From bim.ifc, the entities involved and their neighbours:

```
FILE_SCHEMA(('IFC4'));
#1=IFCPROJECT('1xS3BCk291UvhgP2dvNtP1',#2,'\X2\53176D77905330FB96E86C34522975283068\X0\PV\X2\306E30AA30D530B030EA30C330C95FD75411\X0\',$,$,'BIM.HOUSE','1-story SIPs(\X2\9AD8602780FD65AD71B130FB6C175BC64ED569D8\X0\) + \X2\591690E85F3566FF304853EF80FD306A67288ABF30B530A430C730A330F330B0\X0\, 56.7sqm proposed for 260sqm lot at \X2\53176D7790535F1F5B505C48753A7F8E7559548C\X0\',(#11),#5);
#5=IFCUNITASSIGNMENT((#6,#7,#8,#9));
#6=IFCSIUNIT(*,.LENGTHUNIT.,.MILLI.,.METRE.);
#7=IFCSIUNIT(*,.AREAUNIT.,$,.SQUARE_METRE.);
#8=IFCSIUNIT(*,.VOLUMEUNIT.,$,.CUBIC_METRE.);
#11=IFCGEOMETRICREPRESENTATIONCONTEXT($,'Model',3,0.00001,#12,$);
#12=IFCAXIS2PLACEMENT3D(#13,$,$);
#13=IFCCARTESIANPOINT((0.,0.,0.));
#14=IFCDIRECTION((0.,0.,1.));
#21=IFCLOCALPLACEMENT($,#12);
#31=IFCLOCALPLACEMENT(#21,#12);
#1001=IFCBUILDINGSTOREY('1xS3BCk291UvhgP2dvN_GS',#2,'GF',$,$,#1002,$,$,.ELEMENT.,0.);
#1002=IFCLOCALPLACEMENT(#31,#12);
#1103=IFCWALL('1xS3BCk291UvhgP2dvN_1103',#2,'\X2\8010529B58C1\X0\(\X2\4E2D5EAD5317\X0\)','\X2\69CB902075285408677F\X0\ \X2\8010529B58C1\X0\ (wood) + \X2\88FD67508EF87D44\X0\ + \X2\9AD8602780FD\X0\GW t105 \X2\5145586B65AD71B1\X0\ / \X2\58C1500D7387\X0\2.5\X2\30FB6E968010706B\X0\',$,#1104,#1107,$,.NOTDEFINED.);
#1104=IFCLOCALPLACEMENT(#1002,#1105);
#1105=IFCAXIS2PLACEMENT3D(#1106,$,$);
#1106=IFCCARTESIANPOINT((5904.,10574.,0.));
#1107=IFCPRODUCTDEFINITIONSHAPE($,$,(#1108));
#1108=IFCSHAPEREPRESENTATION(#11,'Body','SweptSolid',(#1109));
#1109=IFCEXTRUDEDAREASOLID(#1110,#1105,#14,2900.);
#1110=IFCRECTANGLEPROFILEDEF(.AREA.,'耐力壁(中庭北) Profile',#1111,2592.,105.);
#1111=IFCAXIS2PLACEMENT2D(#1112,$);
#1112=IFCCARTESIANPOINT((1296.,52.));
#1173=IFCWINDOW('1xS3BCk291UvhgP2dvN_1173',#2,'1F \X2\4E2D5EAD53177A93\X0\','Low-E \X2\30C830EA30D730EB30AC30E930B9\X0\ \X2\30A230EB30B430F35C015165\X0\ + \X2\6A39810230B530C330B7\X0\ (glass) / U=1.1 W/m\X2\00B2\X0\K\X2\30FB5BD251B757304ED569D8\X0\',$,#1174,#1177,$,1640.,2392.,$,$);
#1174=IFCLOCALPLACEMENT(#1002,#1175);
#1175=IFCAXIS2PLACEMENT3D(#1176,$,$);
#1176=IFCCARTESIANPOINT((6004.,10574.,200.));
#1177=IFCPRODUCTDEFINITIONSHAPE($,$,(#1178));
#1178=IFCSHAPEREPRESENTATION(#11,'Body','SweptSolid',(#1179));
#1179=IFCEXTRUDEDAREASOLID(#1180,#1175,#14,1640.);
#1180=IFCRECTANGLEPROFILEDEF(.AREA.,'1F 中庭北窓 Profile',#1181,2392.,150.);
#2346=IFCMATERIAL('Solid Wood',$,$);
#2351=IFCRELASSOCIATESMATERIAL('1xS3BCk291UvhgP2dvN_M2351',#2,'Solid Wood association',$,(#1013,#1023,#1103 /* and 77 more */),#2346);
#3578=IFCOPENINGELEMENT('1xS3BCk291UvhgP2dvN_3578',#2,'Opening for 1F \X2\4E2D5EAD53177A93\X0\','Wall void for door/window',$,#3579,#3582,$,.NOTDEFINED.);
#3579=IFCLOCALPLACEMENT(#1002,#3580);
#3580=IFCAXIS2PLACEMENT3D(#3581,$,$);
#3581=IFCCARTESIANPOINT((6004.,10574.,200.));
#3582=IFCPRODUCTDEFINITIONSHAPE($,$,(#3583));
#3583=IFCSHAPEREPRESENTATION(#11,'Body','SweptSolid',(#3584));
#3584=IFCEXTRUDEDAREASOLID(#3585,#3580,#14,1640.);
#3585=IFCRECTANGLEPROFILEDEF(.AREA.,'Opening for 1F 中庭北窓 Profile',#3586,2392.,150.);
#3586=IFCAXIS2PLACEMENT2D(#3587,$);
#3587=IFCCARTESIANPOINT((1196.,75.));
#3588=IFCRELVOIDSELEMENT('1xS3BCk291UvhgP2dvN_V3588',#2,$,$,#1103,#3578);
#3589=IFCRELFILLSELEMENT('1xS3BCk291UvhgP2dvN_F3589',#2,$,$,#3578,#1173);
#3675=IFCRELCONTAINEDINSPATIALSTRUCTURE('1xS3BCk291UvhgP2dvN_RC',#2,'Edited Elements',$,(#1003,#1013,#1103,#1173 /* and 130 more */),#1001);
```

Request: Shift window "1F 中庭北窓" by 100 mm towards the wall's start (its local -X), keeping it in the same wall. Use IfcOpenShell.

```python
import ifcopenshell
import ifcopenshell.api.geometry
import ifcopenshell.util.placement
import ifcopenshell.util.unit

model = ifcopenshell.open("bim.ifc")
unit_scale = ifcopenshell.util.unit.calculate_unit_scale(model)

window = model.by_guid("1xS3BCk291UvhgP2dvN_1173")
opening = window.FillsVoids[0].RelatingOpeningElement
wall = opening.VoidsElements[0].RelatingBuildingElement

wall_matrix = ifcopenshell.util.placement.get_local_placement(wall.ObjectPlacement)
shift = wall_matrix[:3, 0] * -0.1 / unit_scale
before = ifcopenshell.util.placement.get_local_placement(window.ObjectPlacement)[:3, 3].copy()

# The window is not placed relative to its opening, so move both.
for product in (opening, window):
    matrix = ifcopenshell.util.placement.get_local_placement(product.ObjectPlacement)
    matrix[:3, 3] += shift
    ifcopenshell.api.geometry.edit_object_placement(model, product=product, matrix=matrix, is_si=False)

after = ifcopenshell.util.placement.get_local_placement(window.ObjectPlacement)[:3, 3]
print("window moved by", (after - before).round(3) + 0.0)

model.write("bim_updated.ifc")
```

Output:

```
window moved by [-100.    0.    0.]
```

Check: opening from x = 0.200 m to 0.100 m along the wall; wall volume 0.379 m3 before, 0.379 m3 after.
